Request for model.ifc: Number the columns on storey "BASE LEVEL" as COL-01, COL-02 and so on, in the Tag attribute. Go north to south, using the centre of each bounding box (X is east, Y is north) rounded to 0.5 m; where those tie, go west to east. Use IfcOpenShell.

First a look at what the model holds.

```python
import ifcopenshell
import ifcopenshell.util.element
import ifcopenshell.util.placement

model = ifcopenshell.open("model.ifc")
print(model.schema)
storey = next(s for s in model.by_type("IfcBuildingStorey") if s.Name == "BASE LEVEL")
columns = [e for e in ifcopenshell.util.element.get_decomposition(storey) if e.is_a("IfcColumn")]
for e in sorted(columns, key=lambda e: e.id()):
    origin = ifcopenshell.util.placement.get_local_placement(e.ObjectPlacement)[:3, 3]
    print(e.id(), e.Tag, e.Name, origin.round(2) + 0.0, sep=" | ")
```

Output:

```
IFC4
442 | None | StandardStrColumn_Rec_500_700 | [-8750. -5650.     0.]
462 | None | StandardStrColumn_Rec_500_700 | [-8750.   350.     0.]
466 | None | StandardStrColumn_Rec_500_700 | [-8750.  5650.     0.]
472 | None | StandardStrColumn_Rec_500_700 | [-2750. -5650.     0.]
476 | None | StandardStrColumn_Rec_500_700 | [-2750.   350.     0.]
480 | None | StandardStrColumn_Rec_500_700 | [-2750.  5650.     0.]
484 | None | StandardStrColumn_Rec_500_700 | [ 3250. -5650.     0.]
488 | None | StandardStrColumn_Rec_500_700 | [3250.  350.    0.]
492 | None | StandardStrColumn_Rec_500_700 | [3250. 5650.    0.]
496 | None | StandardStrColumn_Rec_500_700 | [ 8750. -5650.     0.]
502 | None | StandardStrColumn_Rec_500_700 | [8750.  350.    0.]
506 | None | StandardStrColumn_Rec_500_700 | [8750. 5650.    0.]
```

```python
import ifcopenshell
import ifcopenshell.geom
import ifcopenshell.util.element
import ifcopenshell.util.shape

model = ifcopenshell.open("model.ifc")
settings = ifcopenshell.geom.settings()
settings.set("use-world-coords", True)


def centre(element):
    shape = ifcopenshell.geom.create_shape(settings, element)
    return ifcopenshell.util.shape.get_bbox_centroid(shape.geometry)


storey = next(s for s in model.by_type("IfcBuildingStorey") if s.Name == "BASE LEVEL")
columns = [e for e in ifcopenshell.util.element.get_decomposition(storey) if e.is_a("IfcColumn")]

# Insertion points can sit at a corner or the storey origin, so sort by the geometry (in metres).
centres = {e: centre(e) for e in columns}
columns.sort(key=lambda e: (-round(centres[e][1] / 0.5), centres[e][0]))

for i, e in enumerate(columns, start=1):
    number = f"COL-{i:02d}"
    e.Tag = number
    print(e.id(), number)

model.write("model_edited.ifc")
```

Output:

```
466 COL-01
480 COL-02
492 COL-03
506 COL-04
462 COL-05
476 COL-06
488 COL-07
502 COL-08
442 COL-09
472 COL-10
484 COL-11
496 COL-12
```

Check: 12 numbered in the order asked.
